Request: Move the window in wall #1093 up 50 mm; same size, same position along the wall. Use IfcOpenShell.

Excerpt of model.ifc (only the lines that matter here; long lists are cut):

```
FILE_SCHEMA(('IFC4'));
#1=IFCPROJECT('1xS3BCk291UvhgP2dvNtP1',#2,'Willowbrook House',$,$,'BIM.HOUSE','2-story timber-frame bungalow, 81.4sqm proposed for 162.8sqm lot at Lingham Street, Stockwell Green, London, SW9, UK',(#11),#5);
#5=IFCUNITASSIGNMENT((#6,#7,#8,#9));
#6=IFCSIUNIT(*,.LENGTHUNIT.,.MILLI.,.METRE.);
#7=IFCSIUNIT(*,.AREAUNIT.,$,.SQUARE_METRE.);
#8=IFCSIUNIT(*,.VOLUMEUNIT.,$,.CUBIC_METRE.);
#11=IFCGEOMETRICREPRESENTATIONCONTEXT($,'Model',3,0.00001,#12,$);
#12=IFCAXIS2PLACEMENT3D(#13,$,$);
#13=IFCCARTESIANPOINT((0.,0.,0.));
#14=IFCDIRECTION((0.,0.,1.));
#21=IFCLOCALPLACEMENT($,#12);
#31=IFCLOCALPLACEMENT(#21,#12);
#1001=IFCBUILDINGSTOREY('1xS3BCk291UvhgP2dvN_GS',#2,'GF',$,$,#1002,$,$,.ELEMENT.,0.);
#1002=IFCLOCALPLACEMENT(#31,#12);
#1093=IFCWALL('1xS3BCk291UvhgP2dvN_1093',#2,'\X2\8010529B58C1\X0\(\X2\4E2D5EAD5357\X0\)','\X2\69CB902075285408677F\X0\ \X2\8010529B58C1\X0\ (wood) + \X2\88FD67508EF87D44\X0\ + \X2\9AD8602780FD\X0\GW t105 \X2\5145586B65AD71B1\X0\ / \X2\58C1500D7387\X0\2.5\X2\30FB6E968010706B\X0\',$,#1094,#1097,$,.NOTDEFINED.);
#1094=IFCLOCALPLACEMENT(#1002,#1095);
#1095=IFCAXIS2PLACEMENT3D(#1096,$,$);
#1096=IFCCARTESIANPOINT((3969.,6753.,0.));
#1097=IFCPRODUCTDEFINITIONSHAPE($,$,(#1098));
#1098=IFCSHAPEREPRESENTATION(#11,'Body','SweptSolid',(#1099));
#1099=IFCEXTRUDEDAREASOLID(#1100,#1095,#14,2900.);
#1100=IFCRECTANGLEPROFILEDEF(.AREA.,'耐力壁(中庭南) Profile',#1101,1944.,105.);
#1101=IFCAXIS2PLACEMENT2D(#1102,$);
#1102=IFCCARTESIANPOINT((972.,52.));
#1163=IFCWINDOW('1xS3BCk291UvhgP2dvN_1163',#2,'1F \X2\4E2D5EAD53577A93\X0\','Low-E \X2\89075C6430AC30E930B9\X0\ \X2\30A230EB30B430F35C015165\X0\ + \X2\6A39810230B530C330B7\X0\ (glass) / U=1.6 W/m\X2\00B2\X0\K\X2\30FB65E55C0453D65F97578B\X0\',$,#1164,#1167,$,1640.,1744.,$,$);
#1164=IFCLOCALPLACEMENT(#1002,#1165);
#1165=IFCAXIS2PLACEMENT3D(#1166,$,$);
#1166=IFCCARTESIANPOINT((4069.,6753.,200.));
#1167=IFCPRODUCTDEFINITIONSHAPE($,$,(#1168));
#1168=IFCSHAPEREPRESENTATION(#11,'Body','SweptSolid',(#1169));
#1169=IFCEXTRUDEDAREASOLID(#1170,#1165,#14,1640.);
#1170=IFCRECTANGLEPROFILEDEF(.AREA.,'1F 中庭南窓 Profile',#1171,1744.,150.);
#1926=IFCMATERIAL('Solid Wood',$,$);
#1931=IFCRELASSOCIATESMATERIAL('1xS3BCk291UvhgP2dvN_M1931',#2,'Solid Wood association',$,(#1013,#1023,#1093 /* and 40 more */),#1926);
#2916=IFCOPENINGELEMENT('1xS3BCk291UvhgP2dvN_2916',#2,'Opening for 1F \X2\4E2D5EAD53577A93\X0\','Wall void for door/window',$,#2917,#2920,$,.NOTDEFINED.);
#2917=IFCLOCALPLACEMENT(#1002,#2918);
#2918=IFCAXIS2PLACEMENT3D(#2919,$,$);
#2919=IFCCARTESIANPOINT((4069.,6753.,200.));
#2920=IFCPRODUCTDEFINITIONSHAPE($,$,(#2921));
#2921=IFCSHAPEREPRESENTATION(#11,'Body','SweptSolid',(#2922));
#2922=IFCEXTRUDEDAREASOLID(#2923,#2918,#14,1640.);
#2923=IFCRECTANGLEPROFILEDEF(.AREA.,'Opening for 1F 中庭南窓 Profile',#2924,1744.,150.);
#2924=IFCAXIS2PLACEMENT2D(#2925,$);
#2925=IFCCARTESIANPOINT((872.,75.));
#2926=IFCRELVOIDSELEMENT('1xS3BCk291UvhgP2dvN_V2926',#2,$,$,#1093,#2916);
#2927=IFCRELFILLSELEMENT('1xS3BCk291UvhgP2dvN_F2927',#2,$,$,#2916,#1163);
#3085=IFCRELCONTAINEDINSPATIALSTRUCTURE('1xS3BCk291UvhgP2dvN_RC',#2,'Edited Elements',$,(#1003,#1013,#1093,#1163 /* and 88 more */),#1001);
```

```python
import numpy as np
import ifcopenshell
import ifcopenshell.api.geometry
import ifcopenshell.util.placement
import ifcopenshell.util.unit

model = ifcopenshell.open("model.ifc")
unit_scale = ifcopenshell.util.unit.calculate_unit_scale(model)

window = model.by_guid("1xS3BCk291UvhgP2dvN_1163")
opening = window.FillsVoids[0].RelatingOpeningElement
dz = 0.05 / unit_scale

shift = np.array([0.0, 0.0, dz])
# The window is not placed relative to its opening, so move both.
for product in (opening, window):
    matrix = ifcopenshell.util.placement.get_local_placement(product.ObjectPlacement)
    matrix[:3, 3] += shift
    ifcopenshell.api.geometry.edit_object_placement(model, product=product, matrix=matrix, is_si=False)

print(f"moved by {dz * unit_scale:+.3f} m")

model.write("model_rev.ifc")
```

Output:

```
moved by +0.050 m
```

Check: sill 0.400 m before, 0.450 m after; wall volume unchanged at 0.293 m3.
